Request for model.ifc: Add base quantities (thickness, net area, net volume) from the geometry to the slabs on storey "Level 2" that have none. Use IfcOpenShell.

First a look at what the model holds.

```python
import ifcopenshell
import ifcopenshell.util.element
import ifcopenshell.util.unit

model = ifcopenshell.open("model.ifc")
print(model.schema)
for unit_type in ("LENGTHUNIT", "AREAUNIT", "VOLUMEUNIT"):
    print(unit_type, ifcopenshell.util.unit.calculate_unit_scale(model, unit_type))
storey = next(s for s in model.by_type("IfcBuildingStorey") if s.Name == "Level 2")
slabs = [e for e in ifcopenshell.util.element.get_decomposition(storey) if e.is_a("IfcSlab")]
for e in sorted(slabs, key=lambda e: e.id()):
    print(e.id(), e.is_a(), e.Name, list(ifcopenshell.util.element.get_psets(e, qtos_only=True)), sep=" | ")
```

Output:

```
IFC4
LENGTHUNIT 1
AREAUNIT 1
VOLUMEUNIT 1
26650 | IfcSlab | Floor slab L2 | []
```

```python
import ifcopenshell
import ifcopenshell.api.pset
import ifcopenshell.geom
import ifcopenshell.util.element
import ifcopenshell.util.shape
import ifcopenshell.util.unit

model = ifcopenshell.open("model.ifc")
unit_scale = ifcopenshell.util.unit.calculate_unit_scale(model)
area_scale = ifcopenshell.util.unit.calculate_unit_scale(model, "AREAUNIT")
volume_scale = ifcopenshell.util.unit.calculate_unit_scale(model, "VOLUMEUNIT")
settings = ifcopenshell.geom.settings()

storey = next(s for s in model.by_type("IfcBuildingStorey") if s.Name == "Level 2")
slabs = [e for e in ifcopenshell.util.element.get_decomposition(storey) if e.is_a("IfcSlab")]

for e in sorted(slabs, key=lambda e: e.id()):
    if ifcopenshell.util.element.get_psets(e, qtos_only=True, should_inherit=False):
        continue
    # Geometry comes back in metres, in the element's own axes.
    shape = ifcopenshell.geom.create_shape(settings, e)
    values = {
        "Width": ifcopenshell.util.shape.get_z(shape.geometry) / unit_scale,
        "NetArea": ifcopenshell.util.shape.get_footprint_area(shape.geometry) / area_scale,
        "NetVolume": ifcopenshell.util.shape.get_volume(shape.geometry) / volume_scale,
    }
    qto = ifcopenshell.api.pset.add_qto(model, product=e, name="Qto_SlabBaseQuantities")
    ifcopenshell.api.pset.edit_qto(model, qto=qto, properties=values)
    print(e.id(), {k: round(v, 3) for k, v in values.items()})

model.write("model_updated.ifc")
```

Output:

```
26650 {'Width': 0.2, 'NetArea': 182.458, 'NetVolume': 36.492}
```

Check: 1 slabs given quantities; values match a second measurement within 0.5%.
